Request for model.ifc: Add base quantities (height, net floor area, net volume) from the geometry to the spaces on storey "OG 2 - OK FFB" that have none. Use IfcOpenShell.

First a look at what the model holds.

```python
import ifcopenshell
import ifcopenshell.util.element
import ifcopenshell.util.unit

model = ifcopenshell.open("model.ifc")
print(model.schema)
for unit_type in ("LENGTHUNIT", "AREAUNIT", "VOLUMEUNIT"):
    print(unit_type, ifcopenshell.util.unit.calculate_unit_scale(model, unit_type))
storey = next(s for s in model.by_type("IfcBuildingStorey") if s.Name == "OG 2 - OK FFB")
spaces = [e for e in ifcopenshell.util.element.get_decomposition(storey) if e.is_a("IfcSpace")]
for e in sorted(spaces, key=lambda e: e.id()):
    print(e.id(), e.is_a(), e.Name, list(ifcopenshell.util.element.get_psets(e, qtos_only=True)), sep=" | ")
```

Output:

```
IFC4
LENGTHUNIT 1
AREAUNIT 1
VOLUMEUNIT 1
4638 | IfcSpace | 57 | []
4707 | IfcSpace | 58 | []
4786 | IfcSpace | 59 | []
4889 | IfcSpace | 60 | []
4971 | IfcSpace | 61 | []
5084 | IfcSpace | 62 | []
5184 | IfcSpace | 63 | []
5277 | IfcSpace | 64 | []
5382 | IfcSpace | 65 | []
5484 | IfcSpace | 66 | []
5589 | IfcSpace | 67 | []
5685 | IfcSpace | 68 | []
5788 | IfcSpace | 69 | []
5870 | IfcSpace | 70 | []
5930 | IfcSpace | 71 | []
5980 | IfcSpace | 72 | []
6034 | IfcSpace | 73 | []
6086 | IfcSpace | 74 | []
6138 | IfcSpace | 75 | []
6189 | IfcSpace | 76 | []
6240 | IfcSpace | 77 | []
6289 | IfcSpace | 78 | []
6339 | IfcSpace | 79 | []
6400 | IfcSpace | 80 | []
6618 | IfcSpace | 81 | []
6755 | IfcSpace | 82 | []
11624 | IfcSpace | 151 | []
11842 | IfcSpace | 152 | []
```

```python
import ifcopenshell
import ifcopenshell.api.pset
import ifcopenshell.geom
import ifcopenshell.util.element
import ifcopenshell.util.shape
import ifcopenshell.util.unit

model = ifcopenshell.open("model.ifc")
unit_scale = ifcopenshell.util.unit.calculate_unit_scale(model)
area_scale = ifcopenshell.util.unit.calculate_unit_scale(model, "AREAUNIT")
volume_scale = ifcopenshell.util.unit.calculate_unit_scale(model, "VOLUMEUNIT")
settings = ifcopenshell.geom.settings()

storey = next(s for s in model.by_type("IfcBuildingStorey") if s.Name == "OG 2 - OK FFB")
spaces = [e for e in ifcopenshell.util.element.get_decomposition(storey) if e.is_a("IfcSpace")]

for e in sorted(spaces, key=lambda e: e.id()):
    if ifcopenshell.util.element.get_psets(e, qtos_only=True, should_inherit=False):
        continue
    # Geometry comes back in metres, in the element's own axes.
    shape = ifcopenshell.geom.create_shape(settings, e)
    values = {
        "Height": ifcopenshell.util.shape.get_z(shape.geometry) / unit_scale,
        "NetFloorArea": ifcopenshell.util.shape.get_footprint_area(shape.geometry) / area_scale,
        "NetVolume": ifcopenshell.util.shape.get_volume(shape.geometry) / volume_scale,
    }
    qto = ifcopenshell.api.pset.add_qto(model, product=e, name="Qto_SpaceBaseQuantities")
    ifcopenshell.api.pset.edit_qto(model, qto=qto, properties=values)
    print(e.id(), {k: round(v, 3) for k, v in values.items()})

model.write("model_v2.ifc")
```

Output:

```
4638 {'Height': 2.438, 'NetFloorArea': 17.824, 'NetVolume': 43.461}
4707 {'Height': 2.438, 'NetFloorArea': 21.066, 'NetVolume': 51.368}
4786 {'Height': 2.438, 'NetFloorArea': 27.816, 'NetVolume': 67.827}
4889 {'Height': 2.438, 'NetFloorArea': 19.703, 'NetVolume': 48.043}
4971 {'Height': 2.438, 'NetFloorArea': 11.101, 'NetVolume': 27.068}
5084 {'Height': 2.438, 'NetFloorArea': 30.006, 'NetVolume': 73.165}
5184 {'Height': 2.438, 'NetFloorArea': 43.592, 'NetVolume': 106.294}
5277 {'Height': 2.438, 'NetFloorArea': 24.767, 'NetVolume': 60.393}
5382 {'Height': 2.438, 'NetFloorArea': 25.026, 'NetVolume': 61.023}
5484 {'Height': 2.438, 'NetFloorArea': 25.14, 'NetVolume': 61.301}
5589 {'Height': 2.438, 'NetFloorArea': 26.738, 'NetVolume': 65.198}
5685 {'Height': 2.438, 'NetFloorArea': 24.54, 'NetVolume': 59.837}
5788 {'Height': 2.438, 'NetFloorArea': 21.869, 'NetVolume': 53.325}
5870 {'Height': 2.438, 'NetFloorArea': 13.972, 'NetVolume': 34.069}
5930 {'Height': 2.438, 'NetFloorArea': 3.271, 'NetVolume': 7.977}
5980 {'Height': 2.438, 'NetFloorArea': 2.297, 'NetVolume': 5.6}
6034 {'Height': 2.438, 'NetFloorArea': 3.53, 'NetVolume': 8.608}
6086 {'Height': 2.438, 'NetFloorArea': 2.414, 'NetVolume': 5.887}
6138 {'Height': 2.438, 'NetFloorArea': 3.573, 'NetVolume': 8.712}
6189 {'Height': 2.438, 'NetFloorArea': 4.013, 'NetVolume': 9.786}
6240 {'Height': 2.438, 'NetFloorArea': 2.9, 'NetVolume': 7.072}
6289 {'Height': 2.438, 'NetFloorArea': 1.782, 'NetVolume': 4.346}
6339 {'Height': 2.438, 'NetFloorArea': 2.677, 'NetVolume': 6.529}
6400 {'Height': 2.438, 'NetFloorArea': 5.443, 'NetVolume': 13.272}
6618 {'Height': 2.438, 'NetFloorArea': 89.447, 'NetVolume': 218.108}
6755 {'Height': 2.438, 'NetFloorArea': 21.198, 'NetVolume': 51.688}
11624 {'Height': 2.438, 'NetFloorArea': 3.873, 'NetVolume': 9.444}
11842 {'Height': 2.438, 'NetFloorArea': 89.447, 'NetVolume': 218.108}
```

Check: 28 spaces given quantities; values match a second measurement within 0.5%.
